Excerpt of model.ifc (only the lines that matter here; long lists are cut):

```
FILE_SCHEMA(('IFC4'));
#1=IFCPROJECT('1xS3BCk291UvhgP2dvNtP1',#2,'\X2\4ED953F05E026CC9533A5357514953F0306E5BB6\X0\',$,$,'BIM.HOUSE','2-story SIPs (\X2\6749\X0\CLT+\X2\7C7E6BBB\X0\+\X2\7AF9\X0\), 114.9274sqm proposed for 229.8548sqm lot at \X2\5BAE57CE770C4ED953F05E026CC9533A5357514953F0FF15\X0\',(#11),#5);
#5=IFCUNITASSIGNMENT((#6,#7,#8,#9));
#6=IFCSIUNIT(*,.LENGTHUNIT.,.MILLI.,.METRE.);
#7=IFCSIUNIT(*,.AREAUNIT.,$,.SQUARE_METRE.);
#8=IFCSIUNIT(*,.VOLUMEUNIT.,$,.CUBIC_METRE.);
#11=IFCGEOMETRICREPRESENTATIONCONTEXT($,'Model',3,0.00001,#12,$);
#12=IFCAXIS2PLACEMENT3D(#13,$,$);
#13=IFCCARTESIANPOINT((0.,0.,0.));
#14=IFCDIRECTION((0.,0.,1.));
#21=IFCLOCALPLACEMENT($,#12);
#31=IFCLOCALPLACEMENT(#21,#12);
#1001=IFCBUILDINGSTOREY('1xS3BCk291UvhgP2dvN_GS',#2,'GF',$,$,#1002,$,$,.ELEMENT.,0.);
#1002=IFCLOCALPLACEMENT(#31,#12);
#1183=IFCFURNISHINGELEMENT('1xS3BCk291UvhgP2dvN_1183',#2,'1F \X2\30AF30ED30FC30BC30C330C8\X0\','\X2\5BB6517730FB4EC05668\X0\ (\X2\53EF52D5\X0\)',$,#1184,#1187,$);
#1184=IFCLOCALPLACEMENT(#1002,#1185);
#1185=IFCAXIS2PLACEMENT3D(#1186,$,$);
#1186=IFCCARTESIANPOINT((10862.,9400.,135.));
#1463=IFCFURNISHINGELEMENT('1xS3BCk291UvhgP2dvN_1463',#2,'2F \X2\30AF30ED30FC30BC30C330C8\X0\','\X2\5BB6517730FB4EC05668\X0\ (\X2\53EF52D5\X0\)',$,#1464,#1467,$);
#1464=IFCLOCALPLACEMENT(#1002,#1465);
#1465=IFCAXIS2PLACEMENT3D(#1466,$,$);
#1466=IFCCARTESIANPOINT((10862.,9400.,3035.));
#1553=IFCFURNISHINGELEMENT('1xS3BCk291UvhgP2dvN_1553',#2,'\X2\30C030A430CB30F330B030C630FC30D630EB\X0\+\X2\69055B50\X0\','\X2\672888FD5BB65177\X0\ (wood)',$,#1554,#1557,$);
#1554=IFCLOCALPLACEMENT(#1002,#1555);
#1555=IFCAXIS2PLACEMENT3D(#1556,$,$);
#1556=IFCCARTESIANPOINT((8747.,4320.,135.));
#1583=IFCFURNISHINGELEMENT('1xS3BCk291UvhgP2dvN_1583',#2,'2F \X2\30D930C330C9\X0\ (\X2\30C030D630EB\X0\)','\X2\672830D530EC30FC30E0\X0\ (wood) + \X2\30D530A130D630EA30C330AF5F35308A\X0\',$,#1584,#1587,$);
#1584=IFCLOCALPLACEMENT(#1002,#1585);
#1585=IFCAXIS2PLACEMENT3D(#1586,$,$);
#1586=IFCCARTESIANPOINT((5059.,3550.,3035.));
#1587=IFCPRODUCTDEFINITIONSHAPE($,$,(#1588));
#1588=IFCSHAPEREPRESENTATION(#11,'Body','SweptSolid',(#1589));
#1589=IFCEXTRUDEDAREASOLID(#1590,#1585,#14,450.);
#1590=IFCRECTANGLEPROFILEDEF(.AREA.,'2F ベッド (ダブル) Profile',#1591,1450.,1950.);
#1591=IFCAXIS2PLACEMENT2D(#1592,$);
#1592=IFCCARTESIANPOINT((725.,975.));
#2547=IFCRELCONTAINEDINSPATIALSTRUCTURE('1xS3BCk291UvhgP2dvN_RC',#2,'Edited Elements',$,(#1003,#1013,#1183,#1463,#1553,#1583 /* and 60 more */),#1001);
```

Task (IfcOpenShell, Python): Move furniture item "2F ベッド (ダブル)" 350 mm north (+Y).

```python
import ifcopenshell
import ifcopenshell.api.geometry
import ifcopenshell.util.placement
import ifcopenshell.util.unit

model = ifcopenshell.open("model.ifc")
unit_scale = ifcopenshell.util.unit.calculate_unit_scale(model)

item = model.by_id(1583)
matrix = ifcopenshell.util.placement.get_local_placement(item.ObjectPlacement)
matrix[1, 3] += 0.35 / unit_scale
ifcopenshell.api.geometry.edit_object_placement(model, product=item, matrix=matrix, is_si=False)

print(ifcopenshell.util.placement.get_local_placement(item.ObjectPlacement).round(3) + 0.0)

model.write("model_updated.ifc")
```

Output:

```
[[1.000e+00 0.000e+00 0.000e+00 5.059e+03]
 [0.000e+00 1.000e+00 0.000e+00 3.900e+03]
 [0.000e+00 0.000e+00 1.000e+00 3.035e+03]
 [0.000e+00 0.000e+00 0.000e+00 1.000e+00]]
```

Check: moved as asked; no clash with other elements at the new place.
